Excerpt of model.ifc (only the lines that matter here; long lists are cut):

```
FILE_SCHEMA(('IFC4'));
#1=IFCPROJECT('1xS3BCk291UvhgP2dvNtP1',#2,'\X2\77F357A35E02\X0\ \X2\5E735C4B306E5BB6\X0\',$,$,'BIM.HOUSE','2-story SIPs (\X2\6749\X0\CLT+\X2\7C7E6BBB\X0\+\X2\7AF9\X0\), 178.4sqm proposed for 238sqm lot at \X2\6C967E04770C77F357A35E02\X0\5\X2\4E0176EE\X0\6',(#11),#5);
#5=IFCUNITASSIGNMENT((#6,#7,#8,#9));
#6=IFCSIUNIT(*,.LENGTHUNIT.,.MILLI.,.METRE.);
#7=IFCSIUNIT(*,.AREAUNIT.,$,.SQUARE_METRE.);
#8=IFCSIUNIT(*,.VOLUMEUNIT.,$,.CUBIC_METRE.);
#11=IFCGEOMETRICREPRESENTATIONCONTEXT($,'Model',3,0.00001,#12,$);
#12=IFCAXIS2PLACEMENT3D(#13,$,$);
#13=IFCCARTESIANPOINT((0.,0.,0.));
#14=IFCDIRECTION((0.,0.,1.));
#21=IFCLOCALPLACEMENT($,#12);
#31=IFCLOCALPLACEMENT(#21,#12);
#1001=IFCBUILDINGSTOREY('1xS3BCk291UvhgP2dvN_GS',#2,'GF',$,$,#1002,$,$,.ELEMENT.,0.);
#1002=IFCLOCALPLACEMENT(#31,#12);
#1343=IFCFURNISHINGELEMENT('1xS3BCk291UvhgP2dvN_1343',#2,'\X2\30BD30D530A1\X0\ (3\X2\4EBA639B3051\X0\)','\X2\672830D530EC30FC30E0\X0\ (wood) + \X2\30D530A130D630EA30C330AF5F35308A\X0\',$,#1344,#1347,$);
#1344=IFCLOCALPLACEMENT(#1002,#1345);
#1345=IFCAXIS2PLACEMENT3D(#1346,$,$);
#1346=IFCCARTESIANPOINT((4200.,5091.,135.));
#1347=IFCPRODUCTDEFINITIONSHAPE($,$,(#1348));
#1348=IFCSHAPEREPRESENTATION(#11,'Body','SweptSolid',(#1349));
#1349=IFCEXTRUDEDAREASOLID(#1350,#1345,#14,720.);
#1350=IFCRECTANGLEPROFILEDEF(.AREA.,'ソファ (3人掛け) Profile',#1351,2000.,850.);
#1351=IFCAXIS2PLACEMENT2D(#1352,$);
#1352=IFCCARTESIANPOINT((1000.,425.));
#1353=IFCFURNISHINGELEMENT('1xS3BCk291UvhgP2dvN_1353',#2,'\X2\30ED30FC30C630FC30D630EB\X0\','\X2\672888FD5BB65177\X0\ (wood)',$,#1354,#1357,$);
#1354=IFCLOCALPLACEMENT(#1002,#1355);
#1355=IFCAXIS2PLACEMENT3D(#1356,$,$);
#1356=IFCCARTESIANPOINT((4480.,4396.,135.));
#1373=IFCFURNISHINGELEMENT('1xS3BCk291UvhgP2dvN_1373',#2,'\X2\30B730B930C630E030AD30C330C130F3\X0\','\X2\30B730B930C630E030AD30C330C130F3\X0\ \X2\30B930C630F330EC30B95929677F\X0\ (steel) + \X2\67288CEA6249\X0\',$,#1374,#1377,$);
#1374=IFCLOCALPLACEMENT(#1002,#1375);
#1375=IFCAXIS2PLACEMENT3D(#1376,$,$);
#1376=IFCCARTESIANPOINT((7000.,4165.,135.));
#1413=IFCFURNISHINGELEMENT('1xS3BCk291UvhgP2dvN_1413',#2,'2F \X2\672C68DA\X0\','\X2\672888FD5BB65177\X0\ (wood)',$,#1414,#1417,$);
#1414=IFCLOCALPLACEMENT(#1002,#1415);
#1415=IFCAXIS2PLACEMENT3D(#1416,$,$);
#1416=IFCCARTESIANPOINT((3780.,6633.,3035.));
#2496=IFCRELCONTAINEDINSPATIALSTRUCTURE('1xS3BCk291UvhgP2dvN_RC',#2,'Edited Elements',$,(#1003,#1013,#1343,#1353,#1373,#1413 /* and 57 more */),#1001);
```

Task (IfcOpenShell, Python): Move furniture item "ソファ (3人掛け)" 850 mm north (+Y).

```python
import ifcopenshell
import ifcopenshell.api.geometry
import ifcopenshell.util.placement
import ifcopenshell.util.unit

model = ifcopenshell.open("model.ifc")
unit_scale = ifcopenshell.util.unit.calculate_unit_scale(model)

item = model.by_guid("1xS3BCk291UvhgP2dvN_1343")
matrix = ifcopenshell.util.placement.get_local_placement(item.ObjectPlacement)
matrix[1, 3] += 0.85 / unit_scale
ifcopenshell.api.geometry.edit_object_placement(model, product=item, matrix=matrix, is_si=False)

print(ifcopenshell.util.placement.get_local_placement(item.ObjectPlacement).round(3) + 0.0)

model.write("model_edited.ifc")
```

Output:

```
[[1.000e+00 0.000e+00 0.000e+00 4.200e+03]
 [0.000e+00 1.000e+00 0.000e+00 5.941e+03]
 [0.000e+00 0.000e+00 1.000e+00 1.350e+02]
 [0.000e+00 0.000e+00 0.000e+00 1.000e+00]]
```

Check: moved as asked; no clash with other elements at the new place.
